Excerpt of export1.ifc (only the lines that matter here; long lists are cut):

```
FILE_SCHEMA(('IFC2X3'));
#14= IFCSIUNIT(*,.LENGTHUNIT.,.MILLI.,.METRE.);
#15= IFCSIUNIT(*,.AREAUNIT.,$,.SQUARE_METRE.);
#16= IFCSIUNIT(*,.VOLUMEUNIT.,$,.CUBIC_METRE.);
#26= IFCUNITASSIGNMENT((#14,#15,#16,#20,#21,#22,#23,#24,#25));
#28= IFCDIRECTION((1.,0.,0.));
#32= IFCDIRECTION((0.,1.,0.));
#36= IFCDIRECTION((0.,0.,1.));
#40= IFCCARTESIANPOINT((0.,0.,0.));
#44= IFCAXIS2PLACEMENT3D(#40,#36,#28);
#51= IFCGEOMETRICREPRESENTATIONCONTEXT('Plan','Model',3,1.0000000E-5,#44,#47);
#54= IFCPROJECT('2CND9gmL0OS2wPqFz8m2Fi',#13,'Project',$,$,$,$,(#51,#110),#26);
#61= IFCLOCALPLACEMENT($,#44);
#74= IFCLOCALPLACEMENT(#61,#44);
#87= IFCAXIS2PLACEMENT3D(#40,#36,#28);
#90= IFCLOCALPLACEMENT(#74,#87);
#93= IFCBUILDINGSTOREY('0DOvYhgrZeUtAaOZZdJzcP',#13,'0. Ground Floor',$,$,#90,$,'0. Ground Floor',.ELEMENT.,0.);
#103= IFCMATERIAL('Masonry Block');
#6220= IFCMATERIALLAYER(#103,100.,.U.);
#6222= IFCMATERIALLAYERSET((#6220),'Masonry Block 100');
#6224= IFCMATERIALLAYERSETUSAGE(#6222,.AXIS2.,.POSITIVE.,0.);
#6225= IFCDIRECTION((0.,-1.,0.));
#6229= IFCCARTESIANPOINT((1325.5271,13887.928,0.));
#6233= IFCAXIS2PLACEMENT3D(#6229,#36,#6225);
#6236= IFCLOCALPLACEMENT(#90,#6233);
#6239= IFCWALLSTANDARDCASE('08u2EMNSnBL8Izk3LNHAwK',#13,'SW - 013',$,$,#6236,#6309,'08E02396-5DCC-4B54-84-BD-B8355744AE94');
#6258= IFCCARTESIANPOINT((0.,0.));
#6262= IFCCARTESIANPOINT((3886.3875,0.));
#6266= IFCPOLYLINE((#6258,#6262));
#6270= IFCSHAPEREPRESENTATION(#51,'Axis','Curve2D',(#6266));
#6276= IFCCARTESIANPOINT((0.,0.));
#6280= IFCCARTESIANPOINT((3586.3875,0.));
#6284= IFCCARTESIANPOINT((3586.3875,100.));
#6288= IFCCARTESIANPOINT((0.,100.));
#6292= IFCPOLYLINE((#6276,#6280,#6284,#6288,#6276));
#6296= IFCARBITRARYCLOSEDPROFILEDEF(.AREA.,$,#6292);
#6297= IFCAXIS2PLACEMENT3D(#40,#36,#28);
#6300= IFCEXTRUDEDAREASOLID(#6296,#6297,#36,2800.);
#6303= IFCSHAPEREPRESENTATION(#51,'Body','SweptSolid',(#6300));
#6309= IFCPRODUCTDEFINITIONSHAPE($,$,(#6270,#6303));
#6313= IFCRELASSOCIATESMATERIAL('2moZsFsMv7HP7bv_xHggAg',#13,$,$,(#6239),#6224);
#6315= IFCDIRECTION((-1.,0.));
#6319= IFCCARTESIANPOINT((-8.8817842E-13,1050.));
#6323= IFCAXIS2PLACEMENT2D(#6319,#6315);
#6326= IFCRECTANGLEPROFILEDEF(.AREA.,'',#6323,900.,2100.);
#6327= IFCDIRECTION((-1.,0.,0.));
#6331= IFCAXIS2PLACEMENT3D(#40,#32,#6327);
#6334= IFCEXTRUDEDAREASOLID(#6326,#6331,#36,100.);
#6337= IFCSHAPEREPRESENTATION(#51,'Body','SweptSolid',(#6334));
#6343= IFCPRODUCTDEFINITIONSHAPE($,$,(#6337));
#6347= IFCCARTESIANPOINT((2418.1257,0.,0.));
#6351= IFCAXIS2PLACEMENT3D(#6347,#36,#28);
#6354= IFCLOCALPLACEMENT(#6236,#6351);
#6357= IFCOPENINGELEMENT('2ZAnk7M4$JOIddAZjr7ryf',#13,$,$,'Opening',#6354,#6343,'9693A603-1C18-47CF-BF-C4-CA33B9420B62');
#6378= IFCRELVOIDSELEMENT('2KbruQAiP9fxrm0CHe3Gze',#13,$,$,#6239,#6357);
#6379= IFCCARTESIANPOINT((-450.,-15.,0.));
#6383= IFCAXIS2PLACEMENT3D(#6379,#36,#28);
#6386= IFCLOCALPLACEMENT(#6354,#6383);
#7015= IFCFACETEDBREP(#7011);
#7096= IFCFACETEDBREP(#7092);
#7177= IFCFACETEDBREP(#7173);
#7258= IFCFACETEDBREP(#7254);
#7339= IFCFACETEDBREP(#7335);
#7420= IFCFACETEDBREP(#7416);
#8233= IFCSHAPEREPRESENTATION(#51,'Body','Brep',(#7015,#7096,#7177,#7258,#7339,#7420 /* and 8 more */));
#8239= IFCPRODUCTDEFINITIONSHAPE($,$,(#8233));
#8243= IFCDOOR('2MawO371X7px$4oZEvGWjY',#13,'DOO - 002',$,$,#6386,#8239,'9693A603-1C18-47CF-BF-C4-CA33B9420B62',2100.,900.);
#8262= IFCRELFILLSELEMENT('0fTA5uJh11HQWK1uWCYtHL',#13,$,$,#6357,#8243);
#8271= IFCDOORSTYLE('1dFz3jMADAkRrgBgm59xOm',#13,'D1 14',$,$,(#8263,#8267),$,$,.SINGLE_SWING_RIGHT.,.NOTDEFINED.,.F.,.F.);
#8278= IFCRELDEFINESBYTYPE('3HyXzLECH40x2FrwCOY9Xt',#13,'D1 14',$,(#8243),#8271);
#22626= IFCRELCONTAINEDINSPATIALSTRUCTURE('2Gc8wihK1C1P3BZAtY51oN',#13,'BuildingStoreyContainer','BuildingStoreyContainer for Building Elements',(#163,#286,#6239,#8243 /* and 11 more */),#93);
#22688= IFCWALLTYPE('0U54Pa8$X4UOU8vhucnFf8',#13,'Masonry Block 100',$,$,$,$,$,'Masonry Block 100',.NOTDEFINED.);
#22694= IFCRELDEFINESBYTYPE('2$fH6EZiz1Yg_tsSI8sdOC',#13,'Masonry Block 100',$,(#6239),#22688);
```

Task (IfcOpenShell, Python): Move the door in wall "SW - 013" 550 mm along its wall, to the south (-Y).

```python
import ifcopenshell
import ifcopenshell.api.geometry
import ifcopenshell.util.placement

model = ifcopenshell.open("export1.ifc")

door = model.by_id(8243)
opening = door.FillsVoids[0].RelatingOpeningElement
wall = opening.VoidsElements[0].RelatingBuildingElement

wall_matrix = ifcopenshell.util.placement.get_local_placement(wall.ObjectPlacement)
shift = wall_matrix[:3, 0] * 550.0
before = ifcopenshell.util.placement.get_local_placement(door.ObjectPlacement)[:3, 3].copy()

# The door is placed relative to its opening, so it follows when the opening moves.
matrix = ifcopenshell.util.placement.get_local_placement(opening.ObjectPlacement)
matrix[:3, 3] += shift
ifcopenshell.api.geometry.edit_object_placement(
    model, product=opening, matrix=matrix, is_si=False, should_transform_children=True
)

after = ifcopenshell.util.placement.get_local_placement(door.ObjectPlacement)[:3, 3]
print("door moved by", (after - before).round(3) + 0.0)

model.write("export1_edited.ifc")
```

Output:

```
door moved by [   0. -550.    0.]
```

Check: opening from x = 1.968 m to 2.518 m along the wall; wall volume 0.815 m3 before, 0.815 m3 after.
